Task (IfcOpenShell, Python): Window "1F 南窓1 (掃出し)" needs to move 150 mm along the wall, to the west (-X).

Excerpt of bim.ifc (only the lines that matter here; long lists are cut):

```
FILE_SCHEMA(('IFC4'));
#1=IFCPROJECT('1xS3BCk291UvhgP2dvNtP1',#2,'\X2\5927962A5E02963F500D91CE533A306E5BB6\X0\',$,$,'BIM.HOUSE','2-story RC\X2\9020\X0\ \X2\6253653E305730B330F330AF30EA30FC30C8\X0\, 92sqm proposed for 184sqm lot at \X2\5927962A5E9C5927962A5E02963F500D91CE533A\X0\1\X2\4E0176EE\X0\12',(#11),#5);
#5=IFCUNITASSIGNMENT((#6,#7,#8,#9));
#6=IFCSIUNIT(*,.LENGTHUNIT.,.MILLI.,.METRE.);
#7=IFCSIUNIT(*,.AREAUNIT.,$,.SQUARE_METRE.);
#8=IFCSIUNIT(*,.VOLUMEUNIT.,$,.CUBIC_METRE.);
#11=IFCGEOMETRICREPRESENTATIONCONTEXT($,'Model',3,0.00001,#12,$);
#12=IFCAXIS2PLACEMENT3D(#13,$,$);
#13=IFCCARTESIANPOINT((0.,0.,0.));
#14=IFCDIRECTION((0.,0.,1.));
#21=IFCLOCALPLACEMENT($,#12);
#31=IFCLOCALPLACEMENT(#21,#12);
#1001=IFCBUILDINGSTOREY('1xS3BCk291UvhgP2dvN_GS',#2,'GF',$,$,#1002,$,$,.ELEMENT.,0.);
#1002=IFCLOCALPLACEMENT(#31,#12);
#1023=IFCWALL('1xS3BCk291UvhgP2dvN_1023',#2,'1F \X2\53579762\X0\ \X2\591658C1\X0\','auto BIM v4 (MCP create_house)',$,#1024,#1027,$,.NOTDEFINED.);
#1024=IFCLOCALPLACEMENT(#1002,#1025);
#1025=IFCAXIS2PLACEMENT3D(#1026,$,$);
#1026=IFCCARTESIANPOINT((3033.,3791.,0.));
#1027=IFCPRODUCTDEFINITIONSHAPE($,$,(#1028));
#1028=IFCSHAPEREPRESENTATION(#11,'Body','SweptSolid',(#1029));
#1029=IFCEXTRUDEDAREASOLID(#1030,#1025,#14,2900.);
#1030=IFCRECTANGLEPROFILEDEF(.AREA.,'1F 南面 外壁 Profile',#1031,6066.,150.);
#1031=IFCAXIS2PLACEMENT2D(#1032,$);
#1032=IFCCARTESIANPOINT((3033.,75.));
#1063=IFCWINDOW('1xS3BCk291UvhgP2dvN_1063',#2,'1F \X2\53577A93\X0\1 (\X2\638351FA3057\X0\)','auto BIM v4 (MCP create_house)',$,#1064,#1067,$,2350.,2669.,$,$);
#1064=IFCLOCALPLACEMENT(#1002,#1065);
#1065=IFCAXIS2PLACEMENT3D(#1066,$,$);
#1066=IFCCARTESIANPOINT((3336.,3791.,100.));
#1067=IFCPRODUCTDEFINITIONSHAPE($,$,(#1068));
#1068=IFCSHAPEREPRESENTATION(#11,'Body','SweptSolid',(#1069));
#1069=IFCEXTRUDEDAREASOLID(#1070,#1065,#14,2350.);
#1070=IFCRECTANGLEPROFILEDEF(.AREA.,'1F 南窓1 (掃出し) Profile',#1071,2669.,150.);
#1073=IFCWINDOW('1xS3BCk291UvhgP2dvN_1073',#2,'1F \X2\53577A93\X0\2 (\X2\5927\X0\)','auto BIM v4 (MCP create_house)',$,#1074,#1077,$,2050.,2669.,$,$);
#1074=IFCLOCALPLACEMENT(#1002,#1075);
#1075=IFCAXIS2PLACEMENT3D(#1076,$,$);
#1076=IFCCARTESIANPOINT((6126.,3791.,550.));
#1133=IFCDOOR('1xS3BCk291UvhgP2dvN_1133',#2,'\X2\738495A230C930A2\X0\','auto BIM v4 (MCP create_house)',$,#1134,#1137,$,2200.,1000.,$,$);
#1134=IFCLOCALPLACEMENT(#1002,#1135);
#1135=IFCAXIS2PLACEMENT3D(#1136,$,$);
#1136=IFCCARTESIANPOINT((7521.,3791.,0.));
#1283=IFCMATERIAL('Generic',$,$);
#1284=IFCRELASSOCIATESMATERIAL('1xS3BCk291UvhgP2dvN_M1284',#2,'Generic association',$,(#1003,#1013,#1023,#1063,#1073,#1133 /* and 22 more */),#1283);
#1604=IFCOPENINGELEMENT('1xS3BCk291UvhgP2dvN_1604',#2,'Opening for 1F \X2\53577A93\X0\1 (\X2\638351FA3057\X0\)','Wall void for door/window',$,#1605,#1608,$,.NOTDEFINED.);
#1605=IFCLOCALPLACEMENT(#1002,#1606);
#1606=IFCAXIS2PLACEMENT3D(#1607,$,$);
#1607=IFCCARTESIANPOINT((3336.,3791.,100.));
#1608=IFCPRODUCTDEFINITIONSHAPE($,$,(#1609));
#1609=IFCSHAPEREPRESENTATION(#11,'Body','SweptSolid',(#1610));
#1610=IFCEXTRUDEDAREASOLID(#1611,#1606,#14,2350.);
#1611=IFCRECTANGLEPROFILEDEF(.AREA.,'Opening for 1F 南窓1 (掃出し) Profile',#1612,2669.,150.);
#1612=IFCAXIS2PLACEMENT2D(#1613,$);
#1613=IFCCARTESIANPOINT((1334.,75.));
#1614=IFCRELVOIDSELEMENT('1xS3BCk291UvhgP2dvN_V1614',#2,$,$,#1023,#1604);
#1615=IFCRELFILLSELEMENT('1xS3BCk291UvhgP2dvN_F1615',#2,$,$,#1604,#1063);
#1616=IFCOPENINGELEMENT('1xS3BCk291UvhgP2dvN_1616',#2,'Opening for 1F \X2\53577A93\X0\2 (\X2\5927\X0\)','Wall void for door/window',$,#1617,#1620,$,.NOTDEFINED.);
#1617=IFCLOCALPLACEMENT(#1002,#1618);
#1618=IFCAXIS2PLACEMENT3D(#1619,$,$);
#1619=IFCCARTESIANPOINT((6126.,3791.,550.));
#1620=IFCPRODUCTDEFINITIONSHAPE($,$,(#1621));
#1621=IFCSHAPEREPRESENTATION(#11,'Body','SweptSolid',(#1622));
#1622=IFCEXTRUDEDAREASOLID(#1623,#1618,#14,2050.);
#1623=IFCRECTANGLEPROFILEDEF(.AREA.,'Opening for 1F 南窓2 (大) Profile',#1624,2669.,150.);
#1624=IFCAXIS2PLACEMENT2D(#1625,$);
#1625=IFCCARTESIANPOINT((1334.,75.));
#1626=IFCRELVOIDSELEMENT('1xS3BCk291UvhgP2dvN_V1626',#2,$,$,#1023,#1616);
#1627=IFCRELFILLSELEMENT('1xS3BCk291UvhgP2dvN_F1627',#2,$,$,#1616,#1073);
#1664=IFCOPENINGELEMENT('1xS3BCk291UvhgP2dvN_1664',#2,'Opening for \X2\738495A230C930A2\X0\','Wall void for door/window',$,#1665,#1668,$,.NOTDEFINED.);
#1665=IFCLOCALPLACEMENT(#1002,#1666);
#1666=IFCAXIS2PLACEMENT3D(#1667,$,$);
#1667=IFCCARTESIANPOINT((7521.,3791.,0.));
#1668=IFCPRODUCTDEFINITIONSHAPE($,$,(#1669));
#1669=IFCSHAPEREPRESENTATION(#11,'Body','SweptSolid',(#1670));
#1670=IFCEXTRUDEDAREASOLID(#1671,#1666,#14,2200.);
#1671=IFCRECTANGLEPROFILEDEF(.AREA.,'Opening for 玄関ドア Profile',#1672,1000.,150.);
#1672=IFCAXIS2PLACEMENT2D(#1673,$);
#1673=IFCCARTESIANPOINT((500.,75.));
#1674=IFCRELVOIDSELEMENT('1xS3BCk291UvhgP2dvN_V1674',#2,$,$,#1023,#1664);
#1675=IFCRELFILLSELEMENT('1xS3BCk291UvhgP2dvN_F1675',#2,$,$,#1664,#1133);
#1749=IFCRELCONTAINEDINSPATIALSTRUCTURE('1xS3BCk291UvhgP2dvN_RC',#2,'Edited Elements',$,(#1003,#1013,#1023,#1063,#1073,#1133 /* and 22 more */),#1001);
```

```python
import ifcopenshell
import ifcopenshell.api.geometry
import ifcopenshell.util.placement

model = ifcopenshell.open("bim.ifc")

window = model.by_guid("1xS3BCk291UvhgP2dvN_1063")
opening = window.FillsVoids[0].RelatingOpeningElement
wall = opening.VoidsElements[0].RelatingBuildingElement

wall_matrix = ifcopenshell.util.placement.get_local_placement(wall.ObjectPlacement)
shift = wall_matrix[:3, 0] * -150.0
before = ifcopenshell.util.placement.get_local_placement(window.ObjectPlacement)[:3, 3].copy()

# The window is not placed relative to its opening, so move both.
for product in (opening, window):
    matrix = ifcopenshell.util.placement.get_local_placement(product.ObjectPlacement)
    matrix[:3, 3] += shift
    ifcopenshell.api.geometry.edit_object_placement(model, product=product, matrix=matrix, is_si=False)

after = ifcopenshell.util.placement.get_local_placement(window.ObjectPlacement)[:3, 3]
print("window moved by", (after - before).round(3) + 0.0)

model.write("bim_rev.ifc")
```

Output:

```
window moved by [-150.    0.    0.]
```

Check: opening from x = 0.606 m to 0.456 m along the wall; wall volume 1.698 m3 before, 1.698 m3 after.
